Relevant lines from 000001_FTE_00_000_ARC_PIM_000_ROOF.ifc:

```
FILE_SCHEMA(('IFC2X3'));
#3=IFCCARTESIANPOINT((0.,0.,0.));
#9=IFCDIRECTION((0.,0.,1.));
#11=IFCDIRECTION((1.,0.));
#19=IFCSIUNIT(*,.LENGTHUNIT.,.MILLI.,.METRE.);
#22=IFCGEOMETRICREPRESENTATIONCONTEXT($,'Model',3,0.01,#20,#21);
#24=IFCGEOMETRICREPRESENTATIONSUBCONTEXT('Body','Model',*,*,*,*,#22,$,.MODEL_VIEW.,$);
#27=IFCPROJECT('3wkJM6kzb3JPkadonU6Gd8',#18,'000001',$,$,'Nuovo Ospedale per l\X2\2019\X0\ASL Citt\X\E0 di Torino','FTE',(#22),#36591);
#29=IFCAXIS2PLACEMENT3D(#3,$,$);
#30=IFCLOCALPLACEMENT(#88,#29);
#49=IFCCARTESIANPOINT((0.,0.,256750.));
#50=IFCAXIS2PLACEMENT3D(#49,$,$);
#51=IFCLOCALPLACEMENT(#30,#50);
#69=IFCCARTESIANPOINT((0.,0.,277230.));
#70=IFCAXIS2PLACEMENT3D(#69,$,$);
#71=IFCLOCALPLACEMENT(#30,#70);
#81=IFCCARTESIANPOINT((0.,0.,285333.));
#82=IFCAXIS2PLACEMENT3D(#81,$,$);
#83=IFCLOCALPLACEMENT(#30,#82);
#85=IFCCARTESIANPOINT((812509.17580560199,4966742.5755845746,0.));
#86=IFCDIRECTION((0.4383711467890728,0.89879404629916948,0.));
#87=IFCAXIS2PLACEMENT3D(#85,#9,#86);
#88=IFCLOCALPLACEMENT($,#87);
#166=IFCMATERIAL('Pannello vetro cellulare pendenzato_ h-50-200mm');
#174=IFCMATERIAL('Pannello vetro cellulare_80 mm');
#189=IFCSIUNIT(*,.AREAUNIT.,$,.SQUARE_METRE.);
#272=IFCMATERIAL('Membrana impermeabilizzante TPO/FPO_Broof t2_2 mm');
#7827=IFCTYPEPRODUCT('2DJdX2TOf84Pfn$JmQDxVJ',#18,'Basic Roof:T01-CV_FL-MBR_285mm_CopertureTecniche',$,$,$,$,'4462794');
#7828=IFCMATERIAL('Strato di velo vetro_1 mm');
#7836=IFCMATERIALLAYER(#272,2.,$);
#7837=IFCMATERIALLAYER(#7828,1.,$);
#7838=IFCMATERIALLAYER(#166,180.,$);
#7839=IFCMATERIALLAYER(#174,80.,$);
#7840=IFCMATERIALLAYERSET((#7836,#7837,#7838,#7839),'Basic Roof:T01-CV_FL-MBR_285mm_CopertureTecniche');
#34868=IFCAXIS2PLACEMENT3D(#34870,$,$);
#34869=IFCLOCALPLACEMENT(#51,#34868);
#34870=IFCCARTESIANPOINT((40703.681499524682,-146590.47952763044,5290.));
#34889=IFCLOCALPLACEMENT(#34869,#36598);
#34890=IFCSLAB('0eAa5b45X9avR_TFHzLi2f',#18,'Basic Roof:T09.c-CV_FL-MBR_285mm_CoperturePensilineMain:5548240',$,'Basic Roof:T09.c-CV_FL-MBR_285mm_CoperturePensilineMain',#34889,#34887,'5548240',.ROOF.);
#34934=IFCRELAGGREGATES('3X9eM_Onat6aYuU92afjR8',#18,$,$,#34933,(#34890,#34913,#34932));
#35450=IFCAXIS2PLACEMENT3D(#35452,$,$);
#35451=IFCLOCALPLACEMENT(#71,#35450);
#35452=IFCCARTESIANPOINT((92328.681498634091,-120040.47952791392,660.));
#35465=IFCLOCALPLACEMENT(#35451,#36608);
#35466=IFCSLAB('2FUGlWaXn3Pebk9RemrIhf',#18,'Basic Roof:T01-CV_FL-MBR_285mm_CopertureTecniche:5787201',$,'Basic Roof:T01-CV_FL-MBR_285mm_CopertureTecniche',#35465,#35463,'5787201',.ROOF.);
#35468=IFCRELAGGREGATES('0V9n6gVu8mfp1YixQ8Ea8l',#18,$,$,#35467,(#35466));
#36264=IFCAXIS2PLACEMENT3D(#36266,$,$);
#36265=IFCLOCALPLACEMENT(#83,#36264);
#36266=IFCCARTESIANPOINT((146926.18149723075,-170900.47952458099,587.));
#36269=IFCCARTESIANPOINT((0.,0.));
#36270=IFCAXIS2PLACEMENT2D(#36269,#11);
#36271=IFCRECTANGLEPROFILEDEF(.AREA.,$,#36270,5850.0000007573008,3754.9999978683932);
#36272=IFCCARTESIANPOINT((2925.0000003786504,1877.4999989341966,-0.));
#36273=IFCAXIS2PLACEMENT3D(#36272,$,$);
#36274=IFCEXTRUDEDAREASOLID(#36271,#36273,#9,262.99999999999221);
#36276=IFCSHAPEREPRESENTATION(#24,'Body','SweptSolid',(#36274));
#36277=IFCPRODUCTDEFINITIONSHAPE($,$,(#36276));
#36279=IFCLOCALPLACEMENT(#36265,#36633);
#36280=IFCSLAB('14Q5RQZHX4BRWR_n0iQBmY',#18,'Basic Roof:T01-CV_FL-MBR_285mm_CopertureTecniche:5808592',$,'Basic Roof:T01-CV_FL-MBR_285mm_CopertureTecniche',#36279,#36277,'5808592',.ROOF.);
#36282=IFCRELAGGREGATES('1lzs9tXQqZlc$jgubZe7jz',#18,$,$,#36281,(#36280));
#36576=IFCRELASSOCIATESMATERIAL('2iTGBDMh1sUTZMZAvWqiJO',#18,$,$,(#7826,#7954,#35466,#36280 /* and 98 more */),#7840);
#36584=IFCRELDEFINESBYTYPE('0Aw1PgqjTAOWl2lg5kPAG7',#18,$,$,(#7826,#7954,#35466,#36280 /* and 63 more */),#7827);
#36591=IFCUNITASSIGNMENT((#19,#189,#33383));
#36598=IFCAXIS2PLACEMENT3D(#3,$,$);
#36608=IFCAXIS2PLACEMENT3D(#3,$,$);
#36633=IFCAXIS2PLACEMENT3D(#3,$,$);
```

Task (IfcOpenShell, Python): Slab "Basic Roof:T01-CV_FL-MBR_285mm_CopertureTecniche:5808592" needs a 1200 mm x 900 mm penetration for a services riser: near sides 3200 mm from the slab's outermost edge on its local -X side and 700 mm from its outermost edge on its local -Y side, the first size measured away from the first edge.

```python
import numpy as np
import ifcopenshell
import ifcopenshell.api.feature
import ifcopenshell.api.geometry
import ifcopenshell.api.root
import ifcopenshell.geom
import ifcopenshell.util.placement
import ifcopenshell.util.representation
import ifcopenshell.util.shape
import ifcopenshell.util.unit

model = ifcopenshell.open("000001_FTE_00_000_ARC_PIM_000_ROOF.ifc")
unit_scale = ifcopenshell.util.unit.calculate_unit_scale(model)
settings = ifcopenshell.geom.settings()


def volume(element):
    """Net volume in cubic metres, openings subtracted."""
    shape = ifcopenshell.geom.create_shape(settings, element)
    return ifcopenshell.util.shape.get_volume(shape.geometry)


slab = model.by_id(36280)
before = volume(slab)

# Extent in the slab's own axes, in metres. The edges named are its -X and -Y sides.
slab_shape = ifcopenshell.geom.create_shape(settings, slab)
vertices = ifcopenshell.util.shape.get_vertices(slab_shape.geometry)
x_min, y_min, bottom = vertices.min(axis=0)
top = vertices[:, 2].max()

opening = ifcopenshell.api.root.create_entity(model, ifc_class="IfcOpeningElement", name="Services riser opening")
context = ifcopenshell.util.representation.get_context(model, "Model", "Body", "MODEL_VIEW")
width, depth = 1.2, 0.9
outline = [(0.0, 0.0), (width, 0.0), (width, depth), (0.0, depth), (0.0, 0.0)]
# Overshoot both faces by 50 mm so the cut is clean.
shape = ifcopenshell.api.geometry.add_slab_representation(
    model, context=context, depth=top - bottom + 0.1, polyline=outline
)
ifcopenshell.api.geometry.assign_representation(model, product=opening, representation=shape)

matrix = ifcopenshell.util.placement.get_local_placement(slab.ObjectPlacement)
matrix[:, 3] = matrix @ np.append(np.array([x_min + 3.2, y_min + 0.7, bottom - 0.05]) / unit_scale, 1.0)
ifcopenshell.api.geometry.edit_object_placement(model, product=opening, matrix=matrix, is_si=False)
ifcopenshell.api.feature.add_feature(model, feature=opening, element=slab)

after = volume(slab)

print(f"slab volume {before:.3f} -> {after:.3f} m3")

model.write("000001_FTE_00_000_ARC_PIM_000_ROOF-out.ifc")
```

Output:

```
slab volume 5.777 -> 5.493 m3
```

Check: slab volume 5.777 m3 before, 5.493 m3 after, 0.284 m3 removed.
